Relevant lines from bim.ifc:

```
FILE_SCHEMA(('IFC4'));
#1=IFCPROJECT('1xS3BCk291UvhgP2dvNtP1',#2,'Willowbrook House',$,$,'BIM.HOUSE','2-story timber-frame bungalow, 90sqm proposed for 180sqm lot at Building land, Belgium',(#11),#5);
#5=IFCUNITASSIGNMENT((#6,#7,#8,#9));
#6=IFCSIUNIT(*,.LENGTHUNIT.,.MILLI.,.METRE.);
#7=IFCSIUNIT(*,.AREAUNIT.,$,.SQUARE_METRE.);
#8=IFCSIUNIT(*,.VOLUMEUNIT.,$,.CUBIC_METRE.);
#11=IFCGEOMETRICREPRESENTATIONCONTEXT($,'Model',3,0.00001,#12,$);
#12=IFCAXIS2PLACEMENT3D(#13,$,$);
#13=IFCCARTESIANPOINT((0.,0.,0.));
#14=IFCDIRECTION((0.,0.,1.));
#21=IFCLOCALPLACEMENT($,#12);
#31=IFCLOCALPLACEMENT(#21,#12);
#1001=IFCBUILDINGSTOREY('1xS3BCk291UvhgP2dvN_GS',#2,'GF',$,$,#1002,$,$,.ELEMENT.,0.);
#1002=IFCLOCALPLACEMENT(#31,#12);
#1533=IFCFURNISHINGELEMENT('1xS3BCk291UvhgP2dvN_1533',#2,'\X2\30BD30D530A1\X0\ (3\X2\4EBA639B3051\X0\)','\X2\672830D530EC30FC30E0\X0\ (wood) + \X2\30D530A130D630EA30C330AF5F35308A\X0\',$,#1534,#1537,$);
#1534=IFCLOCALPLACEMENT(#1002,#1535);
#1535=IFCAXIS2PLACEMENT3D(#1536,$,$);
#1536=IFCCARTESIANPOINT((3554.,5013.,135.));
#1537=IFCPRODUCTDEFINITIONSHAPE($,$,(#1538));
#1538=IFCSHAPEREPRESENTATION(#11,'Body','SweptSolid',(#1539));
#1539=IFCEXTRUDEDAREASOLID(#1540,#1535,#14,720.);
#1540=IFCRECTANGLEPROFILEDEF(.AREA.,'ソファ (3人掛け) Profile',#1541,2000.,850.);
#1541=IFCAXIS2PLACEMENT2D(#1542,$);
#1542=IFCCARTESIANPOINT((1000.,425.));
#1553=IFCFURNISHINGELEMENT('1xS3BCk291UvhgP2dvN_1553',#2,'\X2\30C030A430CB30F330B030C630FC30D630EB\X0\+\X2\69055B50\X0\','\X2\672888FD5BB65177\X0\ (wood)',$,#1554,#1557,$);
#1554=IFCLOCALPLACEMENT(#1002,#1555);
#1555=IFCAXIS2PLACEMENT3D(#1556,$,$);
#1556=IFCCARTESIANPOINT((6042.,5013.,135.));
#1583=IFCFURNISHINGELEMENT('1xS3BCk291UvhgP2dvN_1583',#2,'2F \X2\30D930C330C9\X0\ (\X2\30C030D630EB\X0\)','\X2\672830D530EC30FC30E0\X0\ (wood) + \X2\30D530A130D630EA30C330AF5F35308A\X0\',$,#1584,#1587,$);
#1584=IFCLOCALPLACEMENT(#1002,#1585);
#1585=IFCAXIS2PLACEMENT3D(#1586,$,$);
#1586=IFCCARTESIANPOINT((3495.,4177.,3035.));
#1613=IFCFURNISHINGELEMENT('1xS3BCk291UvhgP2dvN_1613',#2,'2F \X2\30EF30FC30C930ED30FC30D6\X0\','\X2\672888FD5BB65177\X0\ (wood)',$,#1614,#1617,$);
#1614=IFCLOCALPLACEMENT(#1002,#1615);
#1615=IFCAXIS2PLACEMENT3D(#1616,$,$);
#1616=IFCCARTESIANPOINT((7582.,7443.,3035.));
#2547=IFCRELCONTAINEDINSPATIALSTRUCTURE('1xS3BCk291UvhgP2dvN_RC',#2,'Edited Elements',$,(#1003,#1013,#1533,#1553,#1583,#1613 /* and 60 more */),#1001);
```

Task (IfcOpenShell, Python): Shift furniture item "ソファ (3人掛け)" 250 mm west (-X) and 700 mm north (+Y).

```python
import ifcopenshell
import ifcopenshell.api.geometry
import ifcopenshell.util.placement
import ifcopenshell.util.unit

model = ifcopenshell.open("bim.ifc")
unit_scale = ifcopenshell.util.unit.calculate_unit_scale(model)

item = model.by_guid("1xS3BCk291UvhgP2dvN_1533")
matrix = ifcopenshell.util.placement.get_local_placement(item.ObjectPlacement)
matrix[0, 3] -= 0.25 / unit_scale
matrix[1, 3] += 0.7 / unit_scale
ifcopenshell.api.geometry.edit_object_placement(model, product=item, matrix=matrix, is_si=False)

print(ifcopenshell.util.placement.get_local_placement(item.ObjectPlacement).round(3) + 0.0)

model.write("bim_updated.ifc")
```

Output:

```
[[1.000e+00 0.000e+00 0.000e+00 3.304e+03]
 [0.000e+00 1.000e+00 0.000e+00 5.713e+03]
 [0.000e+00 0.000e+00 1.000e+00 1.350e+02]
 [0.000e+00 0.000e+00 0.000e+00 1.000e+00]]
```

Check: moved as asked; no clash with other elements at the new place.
